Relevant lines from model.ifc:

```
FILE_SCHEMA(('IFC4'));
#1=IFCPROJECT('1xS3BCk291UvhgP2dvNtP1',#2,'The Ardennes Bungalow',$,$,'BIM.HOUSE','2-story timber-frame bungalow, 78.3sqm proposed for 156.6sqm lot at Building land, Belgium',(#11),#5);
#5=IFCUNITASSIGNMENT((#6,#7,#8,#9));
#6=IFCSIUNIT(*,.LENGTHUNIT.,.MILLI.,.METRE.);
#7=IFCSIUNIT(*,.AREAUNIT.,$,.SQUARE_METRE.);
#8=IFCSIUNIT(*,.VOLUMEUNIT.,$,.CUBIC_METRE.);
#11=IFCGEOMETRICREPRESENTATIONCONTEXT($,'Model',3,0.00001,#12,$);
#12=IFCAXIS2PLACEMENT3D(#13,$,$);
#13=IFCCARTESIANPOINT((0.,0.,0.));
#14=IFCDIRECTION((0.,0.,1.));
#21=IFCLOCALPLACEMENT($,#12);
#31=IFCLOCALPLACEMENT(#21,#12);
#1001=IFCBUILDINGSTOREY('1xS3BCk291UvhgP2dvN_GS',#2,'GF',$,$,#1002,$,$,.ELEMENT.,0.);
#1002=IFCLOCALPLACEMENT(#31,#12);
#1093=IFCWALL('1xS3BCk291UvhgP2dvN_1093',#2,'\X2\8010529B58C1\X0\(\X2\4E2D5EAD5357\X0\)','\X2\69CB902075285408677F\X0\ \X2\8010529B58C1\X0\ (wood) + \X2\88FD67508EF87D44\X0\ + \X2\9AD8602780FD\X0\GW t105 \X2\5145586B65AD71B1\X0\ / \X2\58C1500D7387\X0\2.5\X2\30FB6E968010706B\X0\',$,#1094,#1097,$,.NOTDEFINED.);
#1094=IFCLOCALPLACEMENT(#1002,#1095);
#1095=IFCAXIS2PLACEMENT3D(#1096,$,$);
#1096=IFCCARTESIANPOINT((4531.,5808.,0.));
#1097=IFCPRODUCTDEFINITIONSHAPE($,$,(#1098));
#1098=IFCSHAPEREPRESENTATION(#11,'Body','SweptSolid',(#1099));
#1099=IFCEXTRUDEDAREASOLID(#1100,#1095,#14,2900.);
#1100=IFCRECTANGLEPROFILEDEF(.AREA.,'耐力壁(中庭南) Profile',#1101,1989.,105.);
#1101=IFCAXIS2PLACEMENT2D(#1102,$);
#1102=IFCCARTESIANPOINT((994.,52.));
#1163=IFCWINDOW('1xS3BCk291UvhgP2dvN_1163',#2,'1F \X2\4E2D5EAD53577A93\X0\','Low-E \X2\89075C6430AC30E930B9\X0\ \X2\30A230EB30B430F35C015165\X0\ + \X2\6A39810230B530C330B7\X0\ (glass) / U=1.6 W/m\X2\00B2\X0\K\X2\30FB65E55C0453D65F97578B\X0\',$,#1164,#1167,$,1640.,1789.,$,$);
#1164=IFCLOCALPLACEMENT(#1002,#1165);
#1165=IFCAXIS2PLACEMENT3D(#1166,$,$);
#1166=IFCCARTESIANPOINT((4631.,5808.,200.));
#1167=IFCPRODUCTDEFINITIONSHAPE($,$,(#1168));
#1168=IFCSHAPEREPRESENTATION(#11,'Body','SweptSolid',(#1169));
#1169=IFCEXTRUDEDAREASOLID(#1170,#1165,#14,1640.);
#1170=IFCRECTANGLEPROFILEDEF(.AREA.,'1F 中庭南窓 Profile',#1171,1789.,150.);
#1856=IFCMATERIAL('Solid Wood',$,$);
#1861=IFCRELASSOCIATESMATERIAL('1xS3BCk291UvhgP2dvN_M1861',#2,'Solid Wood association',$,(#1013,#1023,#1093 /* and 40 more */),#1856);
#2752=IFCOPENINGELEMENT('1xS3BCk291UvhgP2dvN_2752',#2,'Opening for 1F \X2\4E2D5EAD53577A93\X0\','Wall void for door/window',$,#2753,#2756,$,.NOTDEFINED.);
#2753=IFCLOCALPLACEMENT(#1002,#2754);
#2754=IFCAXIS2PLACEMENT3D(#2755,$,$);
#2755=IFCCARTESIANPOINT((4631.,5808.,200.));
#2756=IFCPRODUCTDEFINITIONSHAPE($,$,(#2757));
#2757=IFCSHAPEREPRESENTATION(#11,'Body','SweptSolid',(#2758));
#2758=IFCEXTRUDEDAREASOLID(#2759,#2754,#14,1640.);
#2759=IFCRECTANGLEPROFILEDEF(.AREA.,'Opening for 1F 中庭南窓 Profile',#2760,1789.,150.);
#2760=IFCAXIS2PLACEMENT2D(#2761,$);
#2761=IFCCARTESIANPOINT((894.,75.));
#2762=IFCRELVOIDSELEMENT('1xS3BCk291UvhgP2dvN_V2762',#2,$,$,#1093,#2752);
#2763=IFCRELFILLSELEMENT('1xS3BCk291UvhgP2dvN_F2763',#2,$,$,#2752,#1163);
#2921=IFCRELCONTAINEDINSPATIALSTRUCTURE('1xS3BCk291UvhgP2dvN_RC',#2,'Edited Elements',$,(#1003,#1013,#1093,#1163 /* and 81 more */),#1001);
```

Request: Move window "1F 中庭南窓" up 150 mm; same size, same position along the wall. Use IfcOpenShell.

```python
import numpy as np
import ifcopenshell
import ifcopenshell.api.geometry
import ifcopenshell.util.placement
import ifcopenshell.util.unit

model = ifcopenshell.open("model.ifc")
unit_scale = ifcopenshell.util.unit.calculate_unit_scale(model)

window = model.by_guid("1xS3BCk291UvhgP2dvN_1163")
opening = window.FillsVoids[0].RelatingOpeningElement
dz = 0.15 / unit_scale

shift = np.array([0.0, 0.0, dz])
# The window is not placed relative to its opening, so move both.
for product in (opening, window):
    matrix = ifcopenshell.util.placement.get_local_placement(product.ObjectPlacement)
    matrix[:3, 3] += shift
    ifcopenshell.api.geometry.edit_object_placement(model, product=product, matrix=matrix, is_si=False)

print(f"moved by {dz * unit_scale:+.3f} m")

model.write("model_v2.ifc")
```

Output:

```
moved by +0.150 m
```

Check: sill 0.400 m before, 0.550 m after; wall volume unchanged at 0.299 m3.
